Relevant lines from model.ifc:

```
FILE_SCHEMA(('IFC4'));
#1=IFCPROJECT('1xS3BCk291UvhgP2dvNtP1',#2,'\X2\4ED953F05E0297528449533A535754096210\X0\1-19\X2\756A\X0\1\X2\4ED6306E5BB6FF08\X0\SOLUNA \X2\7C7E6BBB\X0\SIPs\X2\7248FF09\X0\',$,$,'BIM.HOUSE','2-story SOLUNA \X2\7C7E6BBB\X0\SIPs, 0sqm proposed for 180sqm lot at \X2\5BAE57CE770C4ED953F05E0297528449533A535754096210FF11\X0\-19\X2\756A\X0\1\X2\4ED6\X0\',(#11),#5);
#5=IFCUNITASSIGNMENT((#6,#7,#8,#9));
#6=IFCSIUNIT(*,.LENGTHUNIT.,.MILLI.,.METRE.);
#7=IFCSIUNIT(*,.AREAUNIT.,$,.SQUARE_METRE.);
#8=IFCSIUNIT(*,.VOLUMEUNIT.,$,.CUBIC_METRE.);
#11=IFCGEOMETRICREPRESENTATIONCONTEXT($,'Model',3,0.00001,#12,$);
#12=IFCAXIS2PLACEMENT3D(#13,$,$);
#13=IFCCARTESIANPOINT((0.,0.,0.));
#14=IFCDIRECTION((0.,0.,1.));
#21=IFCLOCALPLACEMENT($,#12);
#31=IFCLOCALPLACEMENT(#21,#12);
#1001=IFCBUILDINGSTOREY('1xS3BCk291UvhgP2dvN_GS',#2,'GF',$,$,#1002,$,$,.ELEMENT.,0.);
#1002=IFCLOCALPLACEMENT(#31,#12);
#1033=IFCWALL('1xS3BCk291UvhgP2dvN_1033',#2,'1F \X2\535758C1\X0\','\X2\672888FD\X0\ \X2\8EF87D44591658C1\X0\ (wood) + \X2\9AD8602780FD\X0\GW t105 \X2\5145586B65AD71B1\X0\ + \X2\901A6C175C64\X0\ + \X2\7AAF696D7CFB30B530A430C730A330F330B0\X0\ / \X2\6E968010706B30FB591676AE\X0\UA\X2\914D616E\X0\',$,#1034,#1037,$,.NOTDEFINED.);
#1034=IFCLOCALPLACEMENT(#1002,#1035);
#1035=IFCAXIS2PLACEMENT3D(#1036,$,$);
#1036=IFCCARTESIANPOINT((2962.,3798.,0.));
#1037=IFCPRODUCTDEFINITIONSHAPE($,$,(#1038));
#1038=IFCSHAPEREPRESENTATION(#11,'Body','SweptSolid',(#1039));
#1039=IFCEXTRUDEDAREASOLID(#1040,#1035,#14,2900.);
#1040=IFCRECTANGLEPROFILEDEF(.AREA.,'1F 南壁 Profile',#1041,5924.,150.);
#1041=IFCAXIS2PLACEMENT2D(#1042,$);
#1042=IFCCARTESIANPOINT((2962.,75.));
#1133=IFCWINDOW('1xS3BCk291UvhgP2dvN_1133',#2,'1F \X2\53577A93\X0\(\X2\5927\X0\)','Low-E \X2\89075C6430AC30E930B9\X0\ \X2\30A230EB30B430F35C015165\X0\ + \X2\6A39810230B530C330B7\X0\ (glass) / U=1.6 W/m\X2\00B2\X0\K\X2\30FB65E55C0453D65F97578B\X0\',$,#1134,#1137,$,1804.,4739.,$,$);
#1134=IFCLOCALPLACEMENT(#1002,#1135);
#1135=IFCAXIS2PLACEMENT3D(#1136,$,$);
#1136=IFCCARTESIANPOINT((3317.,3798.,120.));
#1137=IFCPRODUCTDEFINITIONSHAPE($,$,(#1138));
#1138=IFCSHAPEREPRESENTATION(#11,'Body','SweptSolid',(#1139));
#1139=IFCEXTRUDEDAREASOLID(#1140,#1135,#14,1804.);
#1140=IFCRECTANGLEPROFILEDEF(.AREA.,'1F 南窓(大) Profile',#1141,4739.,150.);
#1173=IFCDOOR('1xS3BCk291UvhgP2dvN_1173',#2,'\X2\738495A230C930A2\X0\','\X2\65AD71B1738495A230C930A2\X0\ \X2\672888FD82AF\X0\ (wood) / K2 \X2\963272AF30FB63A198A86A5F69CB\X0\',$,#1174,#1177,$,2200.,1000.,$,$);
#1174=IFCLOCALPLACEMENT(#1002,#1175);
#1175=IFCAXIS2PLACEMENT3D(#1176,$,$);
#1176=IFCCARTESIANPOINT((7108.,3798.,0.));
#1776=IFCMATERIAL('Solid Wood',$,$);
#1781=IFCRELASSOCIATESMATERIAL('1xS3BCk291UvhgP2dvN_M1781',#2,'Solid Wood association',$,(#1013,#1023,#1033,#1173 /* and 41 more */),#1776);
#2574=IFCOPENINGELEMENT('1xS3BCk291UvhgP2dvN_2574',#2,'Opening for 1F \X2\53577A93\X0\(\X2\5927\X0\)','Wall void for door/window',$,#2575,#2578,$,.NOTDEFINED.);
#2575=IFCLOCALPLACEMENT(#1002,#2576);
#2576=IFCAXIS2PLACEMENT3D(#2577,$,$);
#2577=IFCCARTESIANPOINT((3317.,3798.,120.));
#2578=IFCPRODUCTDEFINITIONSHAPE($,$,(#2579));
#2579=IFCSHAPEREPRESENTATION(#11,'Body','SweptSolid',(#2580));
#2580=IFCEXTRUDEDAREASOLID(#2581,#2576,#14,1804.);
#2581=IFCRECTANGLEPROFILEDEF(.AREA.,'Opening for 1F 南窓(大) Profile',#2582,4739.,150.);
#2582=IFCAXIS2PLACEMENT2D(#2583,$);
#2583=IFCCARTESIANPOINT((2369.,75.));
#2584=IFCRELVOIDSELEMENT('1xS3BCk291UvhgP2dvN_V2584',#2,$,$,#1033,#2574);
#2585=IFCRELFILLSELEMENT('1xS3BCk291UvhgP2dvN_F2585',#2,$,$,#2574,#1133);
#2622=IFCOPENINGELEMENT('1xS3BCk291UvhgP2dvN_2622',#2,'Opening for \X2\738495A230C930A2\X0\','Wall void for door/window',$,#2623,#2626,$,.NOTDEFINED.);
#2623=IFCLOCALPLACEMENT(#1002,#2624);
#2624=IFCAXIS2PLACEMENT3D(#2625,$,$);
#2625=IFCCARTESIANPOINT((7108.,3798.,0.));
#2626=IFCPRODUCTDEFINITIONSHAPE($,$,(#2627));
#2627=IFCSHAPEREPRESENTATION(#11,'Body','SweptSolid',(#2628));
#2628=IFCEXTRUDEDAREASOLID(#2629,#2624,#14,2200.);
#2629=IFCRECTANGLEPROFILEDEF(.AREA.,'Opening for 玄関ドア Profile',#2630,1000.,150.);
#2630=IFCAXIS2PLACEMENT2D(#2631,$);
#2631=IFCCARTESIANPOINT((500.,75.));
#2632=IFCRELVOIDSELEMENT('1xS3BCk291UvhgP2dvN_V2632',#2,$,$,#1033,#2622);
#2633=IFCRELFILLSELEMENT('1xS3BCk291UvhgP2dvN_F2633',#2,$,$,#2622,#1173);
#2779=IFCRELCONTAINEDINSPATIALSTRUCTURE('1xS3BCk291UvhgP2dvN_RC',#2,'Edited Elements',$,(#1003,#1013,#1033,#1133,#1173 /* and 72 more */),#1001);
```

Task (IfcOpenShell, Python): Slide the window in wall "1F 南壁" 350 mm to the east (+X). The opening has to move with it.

```python
import ifcopenshell
import ifcopenshell.api.geometry
import ifcopenshell.util.placement

model = ifcopenshell.open("model.ifc")

window = model.by_guid("1xS3BCk291UvhgP2dvN_1133")
opening = window.FillsVoids[0].RelatingOpeningElement
wall = opening.VoidsElements[0].RelatingBuildingElement

wall_matrix = ifcopenshell.util.placement.get_local_placement(wall.ObjectPlacement)
shift = wall_matrix[:3, 0] * 350.0
before = ifcopenshell.util.placement.get_local_placement(window.ObjectPlacement)[:3, 3].copy()

# The window is not placed relative to its opening, so move both.
for product in (opening, window):
    matrix = ifcopenshell.util.placement.get_local_placement(product.ObjectPlacement)
    matrix[:3, 3] += shift
    ifcopenshell.api.geometry.edit_object_placement(model, product=product, matrix=matrix, is_si=False)

after = ifcopenshell.util.placement.get_local_placement(window.ObjectPlacement)[:3, 3]
print("window moved by", (after - before).round(3) + 0.0)

model.write("model_edited.ifc")
```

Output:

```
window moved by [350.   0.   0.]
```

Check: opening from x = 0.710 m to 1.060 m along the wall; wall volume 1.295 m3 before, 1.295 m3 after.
